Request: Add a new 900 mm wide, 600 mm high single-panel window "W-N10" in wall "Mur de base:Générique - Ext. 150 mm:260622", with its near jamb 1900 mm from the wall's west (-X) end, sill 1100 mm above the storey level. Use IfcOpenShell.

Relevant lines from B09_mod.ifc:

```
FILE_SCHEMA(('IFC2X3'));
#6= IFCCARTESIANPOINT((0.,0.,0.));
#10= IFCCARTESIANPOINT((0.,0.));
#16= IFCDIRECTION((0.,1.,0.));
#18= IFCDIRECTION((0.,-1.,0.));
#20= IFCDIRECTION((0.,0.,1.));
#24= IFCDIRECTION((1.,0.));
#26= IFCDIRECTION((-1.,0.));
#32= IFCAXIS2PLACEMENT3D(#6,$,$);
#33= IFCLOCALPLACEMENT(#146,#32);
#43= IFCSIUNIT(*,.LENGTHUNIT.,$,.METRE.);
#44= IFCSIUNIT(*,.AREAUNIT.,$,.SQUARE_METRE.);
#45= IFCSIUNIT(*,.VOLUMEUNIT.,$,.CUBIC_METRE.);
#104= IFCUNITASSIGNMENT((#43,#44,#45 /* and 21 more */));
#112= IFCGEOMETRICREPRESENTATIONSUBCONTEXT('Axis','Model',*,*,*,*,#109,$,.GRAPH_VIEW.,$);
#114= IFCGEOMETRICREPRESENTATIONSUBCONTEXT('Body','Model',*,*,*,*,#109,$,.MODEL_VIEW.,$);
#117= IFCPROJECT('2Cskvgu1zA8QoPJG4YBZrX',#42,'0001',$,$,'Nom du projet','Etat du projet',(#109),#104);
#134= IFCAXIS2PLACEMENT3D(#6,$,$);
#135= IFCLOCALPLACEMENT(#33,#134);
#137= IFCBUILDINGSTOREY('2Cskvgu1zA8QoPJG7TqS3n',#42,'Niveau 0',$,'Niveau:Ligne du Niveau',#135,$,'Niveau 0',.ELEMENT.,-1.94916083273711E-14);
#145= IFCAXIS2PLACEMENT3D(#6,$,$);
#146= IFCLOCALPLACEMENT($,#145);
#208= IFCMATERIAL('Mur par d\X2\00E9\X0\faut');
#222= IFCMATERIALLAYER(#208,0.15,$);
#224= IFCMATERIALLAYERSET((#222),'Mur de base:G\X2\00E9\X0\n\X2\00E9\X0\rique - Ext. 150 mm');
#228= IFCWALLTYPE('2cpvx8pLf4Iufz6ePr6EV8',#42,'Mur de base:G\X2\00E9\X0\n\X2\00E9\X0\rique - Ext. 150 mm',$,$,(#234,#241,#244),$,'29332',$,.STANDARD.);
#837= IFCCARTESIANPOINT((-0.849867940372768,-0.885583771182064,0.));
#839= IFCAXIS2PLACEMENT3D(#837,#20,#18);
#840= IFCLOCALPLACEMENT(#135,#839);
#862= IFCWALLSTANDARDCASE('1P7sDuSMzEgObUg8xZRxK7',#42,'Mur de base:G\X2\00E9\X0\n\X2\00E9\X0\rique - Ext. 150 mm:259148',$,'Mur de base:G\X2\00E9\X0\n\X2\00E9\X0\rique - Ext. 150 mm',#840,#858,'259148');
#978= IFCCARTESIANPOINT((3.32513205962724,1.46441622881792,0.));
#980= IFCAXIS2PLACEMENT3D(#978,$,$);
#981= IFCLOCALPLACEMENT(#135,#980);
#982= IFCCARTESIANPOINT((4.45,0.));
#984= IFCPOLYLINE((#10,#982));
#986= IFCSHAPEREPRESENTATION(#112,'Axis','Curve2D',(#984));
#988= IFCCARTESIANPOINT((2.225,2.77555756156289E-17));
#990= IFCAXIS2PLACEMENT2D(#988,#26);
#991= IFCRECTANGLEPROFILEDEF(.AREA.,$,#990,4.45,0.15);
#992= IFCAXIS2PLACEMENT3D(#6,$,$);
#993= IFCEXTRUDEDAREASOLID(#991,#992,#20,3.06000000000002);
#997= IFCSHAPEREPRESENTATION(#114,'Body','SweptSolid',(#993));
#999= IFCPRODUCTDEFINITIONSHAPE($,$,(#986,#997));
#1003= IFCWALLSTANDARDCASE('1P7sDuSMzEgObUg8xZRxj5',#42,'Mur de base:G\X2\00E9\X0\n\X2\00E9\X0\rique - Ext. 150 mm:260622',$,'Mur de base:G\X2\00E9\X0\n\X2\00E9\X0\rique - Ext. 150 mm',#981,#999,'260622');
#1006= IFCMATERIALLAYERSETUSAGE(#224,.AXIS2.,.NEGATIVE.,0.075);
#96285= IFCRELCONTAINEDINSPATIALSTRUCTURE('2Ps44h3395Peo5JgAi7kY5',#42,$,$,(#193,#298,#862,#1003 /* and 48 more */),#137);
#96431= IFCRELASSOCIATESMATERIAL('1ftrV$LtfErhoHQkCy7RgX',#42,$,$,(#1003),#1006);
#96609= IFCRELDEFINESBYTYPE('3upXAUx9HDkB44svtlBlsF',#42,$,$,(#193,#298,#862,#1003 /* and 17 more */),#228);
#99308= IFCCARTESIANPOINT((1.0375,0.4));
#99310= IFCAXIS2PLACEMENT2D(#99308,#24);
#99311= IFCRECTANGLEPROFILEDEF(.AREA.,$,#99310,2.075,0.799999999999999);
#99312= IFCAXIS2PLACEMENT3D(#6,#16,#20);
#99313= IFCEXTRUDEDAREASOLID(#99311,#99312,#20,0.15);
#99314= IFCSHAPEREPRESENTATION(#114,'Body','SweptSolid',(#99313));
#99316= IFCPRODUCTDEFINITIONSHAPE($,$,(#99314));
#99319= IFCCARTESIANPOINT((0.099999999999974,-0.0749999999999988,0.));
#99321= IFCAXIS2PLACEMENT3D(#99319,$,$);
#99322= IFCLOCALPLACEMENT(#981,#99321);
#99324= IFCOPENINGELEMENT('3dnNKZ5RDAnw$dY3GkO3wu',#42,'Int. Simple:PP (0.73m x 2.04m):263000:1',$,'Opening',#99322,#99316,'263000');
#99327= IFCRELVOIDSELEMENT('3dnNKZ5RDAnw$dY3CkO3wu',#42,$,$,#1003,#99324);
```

```python
import numpy as np
import ifcopenshell
import ifcopenshell.api.feature
import ifcopenshell.api.geometry
import ifcopenshell.api.root
import ifcopenshell.api.spatial
import ifcopenshell.api.type
import ifcopenshell.geom
import ifcopenshell.util.element
import ifcopenshell.util.placement
import ifcopenshell.util.representation
import ifcopenshell.util.shape
import ifcopenshell.util.unit

model = ifcopenshell.open("B09_mod.ifc")
unit_scale = ifcopenshell.util.unit.calculate_unit_scale(model)
settings = ifcopenshell.geom.settings()


def volume(element):
    """Net volume in cubic metres, openings subtracted."""
    shape = ifcopenshell.geom.create_shape(settings, element)
    return ifcopenshell.util.shape.get_volume(shape.geometry)


wall = model.by_guid("1P7sDuSMzEgObUg8xZRxj5")
storey = ifcopenshell.util.element.get_container(wall, ifc_class="IfcBuildingStorey")
context = ifcopenshell.util.representation.get_context(model, "Model", "Body", "MODEL_VIEW")
before = volume(wall)

width, height, from_end, sill = 0.9, 0.6, 1.9, 1.1  # metres

# The wall runs along its own X axis, and the end named is its -X end.
wall_shape = ifcopenshell.geom.create_shape(settings, wall)
x, y, z = ifcopenshell.util.shape.get_vertices(wall_shape.geometry).T
start = x.min() + from_end
face, thickness = float(y.min()), float(y.max() - y.min())
wall_matrix = ifcopenshell.util.placement.get_local_placement(wall.ObjectPlacement)
level = ifcopenshell.util.placement.get_local_placement(storey.ObjectPlacement)[2, 3]


def in_wall(x, y):
    """Placement at x, y metres in the wall's axes, at sill height."""
    matrix = wall_matrix.copy()
    matrix[:, 3] = wall_matrix @ np.array([x / unit_scale, y / unit_scale, 0.0, 1.0])
    matrix[2, 3] = level + sill / unit_scale
    return matrix


# Opening: a box that overshoots both wall faces by 50 mm.
opening = ifcopenshell.api.root.create_entity(model, ifc_class="IfcOpeningElement")
box = ifcopenshell.api.geometry.add_wall_representation(
    model, context=context, length=width, height=height, thickness=thickness + 0.1
)
ifcopenshell.api.geometry.assign_representation(model, product=opening, representation=box)
ifcopenshell.api.geometry.edit_object_placement(model, product=opening, matrix=in_wall(start, face - 0.05), is_si=False)
ifcopenshell.api.feature.add_feature(model, feature=opening, element=wall)

window = ifcopenshell.api.root.create_entity(model, ifc_class="IfcWindow", name="W-N10")
window.OverallWidth, window.OverallHeight = width / unit_scale, height / unit_scale
body = ifcopenshell.api.geometry.add_window_representation(
    model,
    context=context,
    overall_width=window.OverallWidth,
    overall_height=window.OverallHeight,
    partition_type="SINGLE_PANEL",
)
ifcopenshell.api.geometry.assign_representation(model, product=window, representation=body)
ifcopenshell.api.spatial.assign_container(model, products=[window], relating_structure=storey)
fills = ifcopenshell.api.feature.add_filling(model, opening=opening, element=window)
fills.OwnerHistory = window.OwnerHistory  # required in IFC2X3

# IFC2X3 keeps the operation on the window style.
style = ifcopenshell.api.root.create_entity(model, ifc_class="IfcWindowStyle", name="W-N10")
style.OperationType, style.ConstructionType = "SINGLE_PANEL", "NOTDEFINED"
style.ParameterTakesPrecedence = style.Sizeable = False
ifcopenshell.api.type.assign_type(model, related_objects=[window], relating_type=style)

# Centre the window in the wall's thickness.
ifcopenshell.api.geometry.edit_object_placement(model, product=window, matrix=in_wall(start, face), is_si=False)
window_shape = ifcopenshell.geom.create_shape(settings, window)
depth = ifcopenshell.util.shape.get_vertices(window_shape.geometry)[:, 1]
offset = face + thickness / 2 - (depth.min() + depth.max()) / 2
ifcopenshell.api.geometry.edit_object_placement(model, product=window, matrix=in_wall(start, offset), is_si=False)

after = volume(wall)

print(f"wall volume {before:.3f} -> {after:.3f} m3")

model.write("B09_mod_updated.ifc")
```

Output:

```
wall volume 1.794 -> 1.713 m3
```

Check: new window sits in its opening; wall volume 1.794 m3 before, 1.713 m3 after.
